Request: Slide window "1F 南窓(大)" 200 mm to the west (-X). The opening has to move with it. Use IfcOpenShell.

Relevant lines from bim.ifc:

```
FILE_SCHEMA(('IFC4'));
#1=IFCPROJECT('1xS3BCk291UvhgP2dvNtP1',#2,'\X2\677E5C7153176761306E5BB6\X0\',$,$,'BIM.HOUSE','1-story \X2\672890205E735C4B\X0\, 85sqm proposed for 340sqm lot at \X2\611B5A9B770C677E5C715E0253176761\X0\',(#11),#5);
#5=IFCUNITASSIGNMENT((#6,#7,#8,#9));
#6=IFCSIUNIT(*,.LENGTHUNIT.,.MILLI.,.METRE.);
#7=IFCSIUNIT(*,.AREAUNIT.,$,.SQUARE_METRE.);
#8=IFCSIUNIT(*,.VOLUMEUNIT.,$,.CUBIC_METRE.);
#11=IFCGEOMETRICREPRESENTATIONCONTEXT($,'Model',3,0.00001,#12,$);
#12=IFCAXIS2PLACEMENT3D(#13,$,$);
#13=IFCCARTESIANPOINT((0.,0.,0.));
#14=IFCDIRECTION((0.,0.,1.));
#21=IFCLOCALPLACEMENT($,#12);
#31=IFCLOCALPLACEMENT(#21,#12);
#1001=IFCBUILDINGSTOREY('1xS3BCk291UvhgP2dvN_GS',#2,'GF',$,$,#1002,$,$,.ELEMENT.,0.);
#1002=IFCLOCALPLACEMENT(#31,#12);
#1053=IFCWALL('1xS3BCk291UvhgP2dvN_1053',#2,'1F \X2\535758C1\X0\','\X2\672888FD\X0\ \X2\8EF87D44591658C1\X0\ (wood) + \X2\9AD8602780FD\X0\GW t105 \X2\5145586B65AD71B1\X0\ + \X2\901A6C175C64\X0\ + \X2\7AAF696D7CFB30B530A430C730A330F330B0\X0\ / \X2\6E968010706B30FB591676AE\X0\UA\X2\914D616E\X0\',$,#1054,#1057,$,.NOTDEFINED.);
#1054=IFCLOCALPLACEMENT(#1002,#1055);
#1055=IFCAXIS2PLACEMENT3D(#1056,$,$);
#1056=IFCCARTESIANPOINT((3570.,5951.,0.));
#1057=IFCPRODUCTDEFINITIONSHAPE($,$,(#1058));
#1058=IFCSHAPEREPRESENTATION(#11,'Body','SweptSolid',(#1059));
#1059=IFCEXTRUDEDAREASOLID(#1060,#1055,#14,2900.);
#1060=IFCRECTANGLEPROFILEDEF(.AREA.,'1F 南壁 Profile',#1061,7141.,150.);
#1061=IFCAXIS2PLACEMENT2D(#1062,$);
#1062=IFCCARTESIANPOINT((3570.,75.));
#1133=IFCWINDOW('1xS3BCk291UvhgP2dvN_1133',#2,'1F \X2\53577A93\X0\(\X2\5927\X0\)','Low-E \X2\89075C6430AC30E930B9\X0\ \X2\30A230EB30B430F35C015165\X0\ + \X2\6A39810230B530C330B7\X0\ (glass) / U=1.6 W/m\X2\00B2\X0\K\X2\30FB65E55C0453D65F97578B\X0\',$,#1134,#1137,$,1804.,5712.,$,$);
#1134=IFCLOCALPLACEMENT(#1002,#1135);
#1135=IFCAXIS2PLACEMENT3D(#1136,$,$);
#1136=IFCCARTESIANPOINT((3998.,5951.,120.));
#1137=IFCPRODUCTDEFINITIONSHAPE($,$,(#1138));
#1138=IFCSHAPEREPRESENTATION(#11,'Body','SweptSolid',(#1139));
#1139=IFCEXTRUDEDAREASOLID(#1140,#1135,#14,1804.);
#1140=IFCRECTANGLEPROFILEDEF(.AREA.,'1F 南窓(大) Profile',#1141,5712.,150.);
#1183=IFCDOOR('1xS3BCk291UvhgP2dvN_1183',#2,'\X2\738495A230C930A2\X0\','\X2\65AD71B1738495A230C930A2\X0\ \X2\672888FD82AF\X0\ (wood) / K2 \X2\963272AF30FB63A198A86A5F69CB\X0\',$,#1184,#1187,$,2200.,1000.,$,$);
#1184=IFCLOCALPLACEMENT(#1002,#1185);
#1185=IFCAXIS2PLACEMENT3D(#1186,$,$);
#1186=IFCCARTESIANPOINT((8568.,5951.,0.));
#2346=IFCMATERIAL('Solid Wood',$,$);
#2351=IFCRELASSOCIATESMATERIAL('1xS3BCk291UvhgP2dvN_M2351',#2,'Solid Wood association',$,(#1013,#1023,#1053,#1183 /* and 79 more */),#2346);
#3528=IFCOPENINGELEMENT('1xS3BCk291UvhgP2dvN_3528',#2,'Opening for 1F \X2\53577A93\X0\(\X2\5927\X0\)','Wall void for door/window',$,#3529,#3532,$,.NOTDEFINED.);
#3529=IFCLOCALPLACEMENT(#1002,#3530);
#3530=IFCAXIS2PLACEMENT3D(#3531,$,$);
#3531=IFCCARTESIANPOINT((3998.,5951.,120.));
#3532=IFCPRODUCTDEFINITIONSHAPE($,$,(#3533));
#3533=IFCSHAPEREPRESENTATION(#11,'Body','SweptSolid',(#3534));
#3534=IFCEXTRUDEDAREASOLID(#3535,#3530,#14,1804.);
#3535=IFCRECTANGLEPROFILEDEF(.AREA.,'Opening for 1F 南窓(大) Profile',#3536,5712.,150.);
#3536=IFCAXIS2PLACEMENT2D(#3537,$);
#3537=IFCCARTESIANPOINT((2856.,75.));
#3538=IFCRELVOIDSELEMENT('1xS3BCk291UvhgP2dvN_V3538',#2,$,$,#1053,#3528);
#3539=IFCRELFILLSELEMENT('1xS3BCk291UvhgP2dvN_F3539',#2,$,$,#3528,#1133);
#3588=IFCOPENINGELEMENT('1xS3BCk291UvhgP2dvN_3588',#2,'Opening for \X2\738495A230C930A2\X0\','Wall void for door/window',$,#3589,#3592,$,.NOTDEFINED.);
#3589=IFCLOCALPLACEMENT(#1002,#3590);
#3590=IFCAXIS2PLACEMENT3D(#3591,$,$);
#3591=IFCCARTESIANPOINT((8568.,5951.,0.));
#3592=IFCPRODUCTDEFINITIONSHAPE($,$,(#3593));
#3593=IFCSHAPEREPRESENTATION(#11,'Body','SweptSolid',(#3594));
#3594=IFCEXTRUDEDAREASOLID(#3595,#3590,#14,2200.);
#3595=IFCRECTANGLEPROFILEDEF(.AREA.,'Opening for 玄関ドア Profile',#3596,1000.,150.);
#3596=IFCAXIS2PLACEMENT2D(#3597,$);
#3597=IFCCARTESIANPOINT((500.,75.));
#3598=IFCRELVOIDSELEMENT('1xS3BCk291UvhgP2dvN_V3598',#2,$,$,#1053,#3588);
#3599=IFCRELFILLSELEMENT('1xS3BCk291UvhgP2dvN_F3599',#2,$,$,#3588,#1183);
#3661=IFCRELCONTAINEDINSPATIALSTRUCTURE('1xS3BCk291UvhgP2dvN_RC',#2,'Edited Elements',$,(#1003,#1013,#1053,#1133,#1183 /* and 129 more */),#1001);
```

```python
import ifcopenshell
import ifcopenshell.api.geometry
import ifcopenshell.util.placement
import ifcopenshell.util.unit

model = ifcopenshell.open("bim.ifc")
unit_scale = ifcopenshell.util.unit.calculate_unit_scale(model)

window = model.by_id(1133)
opening = window.FillsVoids[0].RelatingOpeningElement
wall = opening.VoidsElements[0].RelatingBuildingElement

wall_matrix = ifcopenshell.util.placement.get_local_placement(wall.ObjectPlacement)
shift = wall_matrix[:3, 0] * -0.2 / unit_scale
before = ifcopenshell.util.placement.get_local_placement(window.ObjectPlacement)[:3, 3].copy()

# The window is not placed relative to its opening, so move both.
for product in (opening, window):
    matrix = ifcopenshell.util.placement.get_local_placement(product.ObjectPlacement)
    matrix[:3, 3] += shift
    ifcopenshell.api.geometry.edit_object_placement(model, product=product, matrix=matrix, is_si=False)

after = ifcopenshell.util.placement.get_local_placement(window.ObjectPlacement)[:3, 3]
print("window moved by", (after - before).round(3) + 0.0)

model.write("bim_rev.ifc")
```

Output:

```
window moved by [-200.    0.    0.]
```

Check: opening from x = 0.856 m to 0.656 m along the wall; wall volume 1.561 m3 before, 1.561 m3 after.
